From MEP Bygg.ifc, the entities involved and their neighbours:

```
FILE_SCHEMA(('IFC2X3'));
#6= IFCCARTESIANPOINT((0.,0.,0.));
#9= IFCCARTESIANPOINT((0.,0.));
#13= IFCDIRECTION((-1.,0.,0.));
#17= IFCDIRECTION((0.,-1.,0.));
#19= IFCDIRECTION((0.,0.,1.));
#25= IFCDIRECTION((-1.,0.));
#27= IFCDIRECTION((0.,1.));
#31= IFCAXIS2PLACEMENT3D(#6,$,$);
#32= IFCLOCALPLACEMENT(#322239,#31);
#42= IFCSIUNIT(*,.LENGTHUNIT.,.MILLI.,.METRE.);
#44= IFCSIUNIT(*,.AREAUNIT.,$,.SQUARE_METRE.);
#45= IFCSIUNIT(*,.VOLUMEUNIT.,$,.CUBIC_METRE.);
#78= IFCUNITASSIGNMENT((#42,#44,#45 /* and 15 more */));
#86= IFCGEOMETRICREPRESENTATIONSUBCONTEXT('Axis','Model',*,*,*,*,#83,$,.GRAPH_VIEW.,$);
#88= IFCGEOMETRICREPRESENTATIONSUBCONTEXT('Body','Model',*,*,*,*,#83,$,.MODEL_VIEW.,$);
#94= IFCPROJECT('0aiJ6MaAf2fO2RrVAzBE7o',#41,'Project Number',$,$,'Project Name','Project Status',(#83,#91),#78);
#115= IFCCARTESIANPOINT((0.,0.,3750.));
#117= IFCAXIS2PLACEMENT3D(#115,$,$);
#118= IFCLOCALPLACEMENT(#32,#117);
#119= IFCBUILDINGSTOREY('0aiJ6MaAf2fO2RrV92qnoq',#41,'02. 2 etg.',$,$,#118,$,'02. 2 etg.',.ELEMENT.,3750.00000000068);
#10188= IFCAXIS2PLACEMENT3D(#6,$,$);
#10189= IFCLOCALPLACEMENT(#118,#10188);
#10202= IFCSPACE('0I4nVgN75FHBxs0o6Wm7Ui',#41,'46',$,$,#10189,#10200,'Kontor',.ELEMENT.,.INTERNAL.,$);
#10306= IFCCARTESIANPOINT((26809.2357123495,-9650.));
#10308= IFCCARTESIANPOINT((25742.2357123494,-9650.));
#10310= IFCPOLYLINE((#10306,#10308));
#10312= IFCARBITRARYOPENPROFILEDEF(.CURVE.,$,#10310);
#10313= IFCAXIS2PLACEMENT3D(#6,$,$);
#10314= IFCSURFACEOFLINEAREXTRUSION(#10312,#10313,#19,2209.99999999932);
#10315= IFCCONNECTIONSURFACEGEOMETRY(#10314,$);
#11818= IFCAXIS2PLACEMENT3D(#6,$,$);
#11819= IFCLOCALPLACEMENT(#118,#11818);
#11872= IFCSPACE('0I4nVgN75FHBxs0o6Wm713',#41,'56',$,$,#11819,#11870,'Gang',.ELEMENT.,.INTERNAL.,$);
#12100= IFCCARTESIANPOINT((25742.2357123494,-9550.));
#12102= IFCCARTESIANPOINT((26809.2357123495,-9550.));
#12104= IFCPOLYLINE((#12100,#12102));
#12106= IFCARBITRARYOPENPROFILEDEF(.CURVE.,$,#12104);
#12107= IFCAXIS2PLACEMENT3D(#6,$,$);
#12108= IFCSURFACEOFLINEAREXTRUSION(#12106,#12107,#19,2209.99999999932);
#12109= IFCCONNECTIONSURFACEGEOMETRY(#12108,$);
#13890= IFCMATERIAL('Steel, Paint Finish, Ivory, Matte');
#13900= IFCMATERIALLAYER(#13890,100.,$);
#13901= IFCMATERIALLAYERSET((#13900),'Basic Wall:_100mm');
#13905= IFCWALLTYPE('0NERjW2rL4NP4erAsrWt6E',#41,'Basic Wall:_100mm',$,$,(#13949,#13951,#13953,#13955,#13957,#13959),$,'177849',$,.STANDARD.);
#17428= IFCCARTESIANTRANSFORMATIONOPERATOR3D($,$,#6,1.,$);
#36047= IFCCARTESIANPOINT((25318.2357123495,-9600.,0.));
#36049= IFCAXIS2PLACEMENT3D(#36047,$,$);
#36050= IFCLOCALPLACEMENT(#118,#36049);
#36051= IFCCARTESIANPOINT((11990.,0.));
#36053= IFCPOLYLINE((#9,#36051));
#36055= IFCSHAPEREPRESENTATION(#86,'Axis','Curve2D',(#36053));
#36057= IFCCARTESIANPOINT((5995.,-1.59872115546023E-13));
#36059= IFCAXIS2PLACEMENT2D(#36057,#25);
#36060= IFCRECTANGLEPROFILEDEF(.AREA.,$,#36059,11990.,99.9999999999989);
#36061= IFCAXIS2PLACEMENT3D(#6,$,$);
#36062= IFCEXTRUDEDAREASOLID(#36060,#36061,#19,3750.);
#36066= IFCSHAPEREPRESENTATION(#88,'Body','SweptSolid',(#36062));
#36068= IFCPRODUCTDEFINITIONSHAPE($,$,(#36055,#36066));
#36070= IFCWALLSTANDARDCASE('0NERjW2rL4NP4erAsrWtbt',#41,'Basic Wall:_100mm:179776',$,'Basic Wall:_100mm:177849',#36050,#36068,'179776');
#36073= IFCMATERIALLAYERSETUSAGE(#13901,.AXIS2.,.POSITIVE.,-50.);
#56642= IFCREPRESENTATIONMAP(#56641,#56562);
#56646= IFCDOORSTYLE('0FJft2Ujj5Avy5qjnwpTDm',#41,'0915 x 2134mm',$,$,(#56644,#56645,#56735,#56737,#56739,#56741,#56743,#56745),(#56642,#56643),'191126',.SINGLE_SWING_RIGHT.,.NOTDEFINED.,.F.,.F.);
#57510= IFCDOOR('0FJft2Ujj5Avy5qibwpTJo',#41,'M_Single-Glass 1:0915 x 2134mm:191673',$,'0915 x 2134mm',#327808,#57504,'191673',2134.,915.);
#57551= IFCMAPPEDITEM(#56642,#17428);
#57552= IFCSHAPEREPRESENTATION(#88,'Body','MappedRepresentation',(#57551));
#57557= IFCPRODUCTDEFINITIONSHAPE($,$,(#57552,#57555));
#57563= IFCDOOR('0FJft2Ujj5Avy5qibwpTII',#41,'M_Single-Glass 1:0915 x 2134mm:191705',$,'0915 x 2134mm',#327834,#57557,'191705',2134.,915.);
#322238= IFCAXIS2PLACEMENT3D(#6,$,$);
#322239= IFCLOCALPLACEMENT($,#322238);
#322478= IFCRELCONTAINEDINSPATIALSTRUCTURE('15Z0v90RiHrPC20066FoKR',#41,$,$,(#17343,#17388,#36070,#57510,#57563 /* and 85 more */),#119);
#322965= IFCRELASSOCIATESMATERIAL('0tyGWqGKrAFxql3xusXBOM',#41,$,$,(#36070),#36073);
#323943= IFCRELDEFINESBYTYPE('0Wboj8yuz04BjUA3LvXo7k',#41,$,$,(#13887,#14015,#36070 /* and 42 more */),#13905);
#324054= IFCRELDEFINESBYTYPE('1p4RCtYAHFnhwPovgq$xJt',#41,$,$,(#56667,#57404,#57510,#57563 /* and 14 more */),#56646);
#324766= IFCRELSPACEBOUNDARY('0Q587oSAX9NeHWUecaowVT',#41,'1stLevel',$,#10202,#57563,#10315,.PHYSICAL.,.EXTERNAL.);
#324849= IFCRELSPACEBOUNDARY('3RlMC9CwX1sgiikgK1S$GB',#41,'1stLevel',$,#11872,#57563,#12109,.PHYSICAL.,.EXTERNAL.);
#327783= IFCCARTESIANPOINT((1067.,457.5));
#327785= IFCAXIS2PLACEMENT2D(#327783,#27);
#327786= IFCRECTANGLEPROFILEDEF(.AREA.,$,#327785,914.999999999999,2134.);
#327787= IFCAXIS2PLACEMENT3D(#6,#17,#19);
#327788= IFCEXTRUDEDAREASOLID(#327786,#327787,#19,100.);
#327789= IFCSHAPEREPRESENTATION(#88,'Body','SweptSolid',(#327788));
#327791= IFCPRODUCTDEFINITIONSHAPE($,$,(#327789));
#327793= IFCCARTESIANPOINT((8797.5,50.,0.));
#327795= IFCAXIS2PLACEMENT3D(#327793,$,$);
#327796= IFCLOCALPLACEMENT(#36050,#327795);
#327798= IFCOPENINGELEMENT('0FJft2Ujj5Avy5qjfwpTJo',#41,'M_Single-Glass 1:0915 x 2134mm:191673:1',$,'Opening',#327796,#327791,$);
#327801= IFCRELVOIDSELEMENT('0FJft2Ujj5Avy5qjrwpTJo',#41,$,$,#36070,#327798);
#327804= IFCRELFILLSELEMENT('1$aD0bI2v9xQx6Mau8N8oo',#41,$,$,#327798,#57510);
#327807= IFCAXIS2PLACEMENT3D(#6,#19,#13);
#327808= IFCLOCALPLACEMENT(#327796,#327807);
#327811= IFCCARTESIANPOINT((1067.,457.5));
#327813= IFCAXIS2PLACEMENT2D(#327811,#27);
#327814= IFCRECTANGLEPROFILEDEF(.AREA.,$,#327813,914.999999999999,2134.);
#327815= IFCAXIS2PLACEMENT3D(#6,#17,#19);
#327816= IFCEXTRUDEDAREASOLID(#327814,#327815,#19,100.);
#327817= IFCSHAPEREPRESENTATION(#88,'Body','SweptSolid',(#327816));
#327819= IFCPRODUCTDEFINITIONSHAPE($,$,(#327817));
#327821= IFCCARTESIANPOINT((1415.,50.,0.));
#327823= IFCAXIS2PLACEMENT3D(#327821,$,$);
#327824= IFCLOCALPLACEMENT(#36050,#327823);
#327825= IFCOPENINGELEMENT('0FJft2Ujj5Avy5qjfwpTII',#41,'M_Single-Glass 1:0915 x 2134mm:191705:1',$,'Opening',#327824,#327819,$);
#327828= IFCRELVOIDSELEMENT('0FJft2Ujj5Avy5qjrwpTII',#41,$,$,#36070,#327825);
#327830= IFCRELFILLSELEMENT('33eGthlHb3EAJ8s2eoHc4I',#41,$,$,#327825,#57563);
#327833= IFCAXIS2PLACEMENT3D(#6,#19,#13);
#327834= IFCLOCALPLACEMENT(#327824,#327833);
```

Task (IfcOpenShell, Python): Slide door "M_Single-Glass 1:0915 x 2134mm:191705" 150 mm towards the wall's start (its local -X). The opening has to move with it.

```python
import numpy as np
import ifcopenshell
import ifcopenshell.api.geometry
import ifcopenshell.util.placement
import ifcopenshell.util.unit

model = ifcopenshell.open("MEP Bygg.ifc")
unit_scale = ifcopenshell.util.unit.calculate_unit_scale(model)

door = model.by_guid("0FJft2Ujj5Avy5qibwpTII")
opening = door.FillsVoids[0].RelatingOpeningElement
wall = opening.VoidsElements[0].RelatingBuildingElement

wall_matrix = ifcopenshell.util.placement.get_local_placement(wall.ObjectPlacement)
shift = wall_matrix[:3, 0] * -0.15 / unit_scale
before = ifcopenshell.util.placement.get_local_placement(door.ObjectPlacement)[:3, 3].copy()

# The door is placed relative to its opening, so it follows when the opening moves.
matrix = ifcopenshell.util.placement.get_local_placement(opening.ObjectPlacement)
matrix[:3, 3] += shift
ifcopenshell.api.geometry.edit_object_placement(
    model, product=opening, matrix=matrix, is_si=False, should_transform_children=True
)

# Space boundary surfaces are stored in each space's coordinates; move them too.
for rel in door.ProvidesBoundaries:
    if not rel.ConnectionGeometry:
        continue
    surface = rel.ConnectionGeometry.SurfaceOnRelatingElement
    space_matrix = ifcopenshell.util.placement.get_local_placement(rel.RelatingSpace.ObjectPlacement)
    point = np.array(surface.Position.Location.Coordinates) + space_matrix[:3, :3].T @ shift
    surface.Position = model.createIfcAxis2Placement3D(
        model.createIfcCartesianPoint(point.tolist()), surface.Position.Axis, surface.Position.RefDirection
    )

after = ifcopenshell.util.placement.get_local_placement(door.ObjectPlacement)[:3, 3]
print("door moved by", (after - before).round(3) + 0.0)

model.write("MEP Bygg_rev.ifc")
```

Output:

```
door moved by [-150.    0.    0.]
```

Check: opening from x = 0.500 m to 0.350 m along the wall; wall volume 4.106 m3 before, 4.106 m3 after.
